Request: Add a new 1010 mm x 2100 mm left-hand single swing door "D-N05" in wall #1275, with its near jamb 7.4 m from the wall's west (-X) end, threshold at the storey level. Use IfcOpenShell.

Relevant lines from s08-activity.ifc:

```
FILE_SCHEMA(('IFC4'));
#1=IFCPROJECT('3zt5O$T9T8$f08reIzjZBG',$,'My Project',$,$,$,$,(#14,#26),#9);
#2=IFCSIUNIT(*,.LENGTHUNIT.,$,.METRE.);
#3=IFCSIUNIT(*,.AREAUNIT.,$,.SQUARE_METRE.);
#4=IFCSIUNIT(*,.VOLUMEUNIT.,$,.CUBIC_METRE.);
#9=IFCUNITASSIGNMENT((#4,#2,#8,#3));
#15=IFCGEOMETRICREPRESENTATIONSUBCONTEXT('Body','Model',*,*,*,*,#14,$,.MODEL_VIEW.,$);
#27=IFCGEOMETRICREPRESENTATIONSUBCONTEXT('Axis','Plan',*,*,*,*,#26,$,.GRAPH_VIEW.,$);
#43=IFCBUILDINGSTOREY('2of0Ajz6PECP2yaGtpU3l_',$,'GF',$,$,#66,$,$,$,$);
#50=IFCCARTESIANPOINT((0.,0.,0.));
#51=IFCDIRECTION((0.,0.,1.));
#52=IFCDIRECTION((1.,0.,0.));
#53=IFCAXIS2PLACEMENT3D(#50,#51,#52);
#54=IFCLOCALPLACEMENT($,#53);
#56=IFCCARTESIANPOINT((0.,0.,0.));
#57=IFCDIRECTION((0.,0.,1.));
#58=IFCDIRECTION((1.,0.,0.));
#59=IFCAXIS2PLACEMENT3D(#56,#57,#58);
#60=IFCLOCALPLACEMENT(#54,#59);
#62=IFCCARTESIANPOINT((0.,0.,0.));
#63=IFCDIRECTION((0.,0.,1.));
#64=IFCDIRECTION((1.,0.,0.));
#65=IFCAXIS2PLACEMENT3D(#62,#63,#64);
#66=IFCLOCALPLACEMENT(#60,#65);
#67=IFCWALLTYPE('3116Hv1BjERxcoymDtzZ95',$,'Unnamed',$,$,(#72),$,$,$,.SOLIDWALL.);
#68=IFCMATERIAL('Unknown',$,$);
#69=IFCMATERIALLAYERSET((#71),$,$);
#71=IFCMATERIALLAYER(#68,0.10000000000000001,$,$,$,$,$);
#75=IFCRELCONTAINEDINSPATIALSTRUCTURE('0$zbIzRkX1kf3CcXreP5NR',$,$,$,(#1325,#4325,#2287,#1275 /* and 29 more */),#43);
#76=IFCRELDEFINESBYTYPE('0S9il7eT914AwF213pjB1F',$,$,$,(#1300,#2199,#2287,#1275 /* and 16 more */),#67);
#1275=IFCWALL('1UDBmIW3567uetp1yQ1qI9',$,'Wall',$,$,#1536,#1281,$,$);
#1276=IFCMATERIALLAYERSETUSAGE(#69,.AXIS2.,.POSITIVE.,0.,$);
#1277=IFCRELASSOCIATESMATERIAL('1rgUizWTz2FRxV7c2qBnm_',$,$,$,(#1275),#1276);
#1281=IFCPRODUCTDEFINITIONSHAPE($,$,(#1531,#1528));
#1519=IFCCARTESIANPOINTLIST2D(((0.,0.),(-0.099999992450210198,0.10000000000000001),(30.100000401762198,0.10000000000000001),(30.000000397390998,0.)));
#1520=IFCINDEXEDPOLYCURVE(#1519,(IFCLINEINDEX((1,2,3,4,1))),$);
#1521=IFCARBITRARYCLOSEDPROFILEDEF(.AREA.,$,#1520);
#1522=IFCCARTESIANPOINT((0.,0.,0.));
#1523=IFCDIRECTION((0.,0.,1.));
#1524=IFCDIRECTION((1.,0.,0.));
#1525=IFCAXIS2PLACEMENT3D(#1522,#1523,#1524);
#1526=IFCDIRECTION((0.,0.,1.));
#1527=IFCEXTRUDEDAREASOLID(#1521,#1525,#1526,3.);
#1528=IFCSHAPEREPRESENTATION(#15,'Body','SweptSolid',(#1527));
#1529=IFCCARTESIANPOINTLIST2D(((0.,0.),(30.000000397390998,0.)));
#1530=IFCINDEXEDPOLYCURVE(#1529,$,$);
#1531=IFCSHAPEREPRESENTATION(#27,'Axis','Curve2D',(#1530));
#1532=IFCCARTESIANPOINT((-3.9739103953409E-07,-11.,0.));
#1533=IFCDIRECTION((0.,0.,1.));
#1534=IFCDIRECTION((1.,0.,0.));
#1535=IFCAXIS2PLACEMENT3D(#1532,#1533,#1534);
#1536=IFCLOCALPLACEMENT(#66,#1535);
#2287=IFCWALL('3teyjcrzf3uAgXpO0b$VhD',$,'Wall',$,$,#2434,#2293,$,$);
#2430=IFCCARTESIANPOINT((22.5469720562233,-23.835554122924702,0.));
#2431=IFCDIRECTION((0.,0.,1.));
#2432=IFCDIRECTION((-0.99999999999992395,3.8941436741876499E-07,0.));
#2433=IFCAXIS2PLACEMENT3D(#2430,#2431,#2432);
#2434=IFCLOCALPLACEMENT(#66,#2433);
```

```python
import numpy as np
import ifcopenshell
import ifcopenshell.api.feature
import ifcopenshell.api.geometry
import ifcopenshell.api.root
import ifcopenshell.api.spatial
import ifcopenshell.geom
import ifcopenshell.util.element
import ifcopenshell.util.placement
import ifcopenshell.util.representation
import ifcopenshell.util.shape
import ifcopenshell.util.unit

model = ifcopenshell.open("s08-activity.ifc")
unit_scale = ifcopenshell.util.unit.calculate_unit_scale(model)
settings = ifcopenshell.geom.settings()


def volume(element):
    """Net volume in cubic metres, openings subtracted."""
    shape = ifcopenshell.geom.create_shape(settings, element)
    return ifcopenshell.util.shape.get_volume(shape.geometry)


wall = model.by_guid("1UDBmIW3567uetp1yQ1qI9")
storey = ifcopenshell.util.element.get_container(wall, ifc_class="IfcBuildingStorey")
context = ifcopenshell.util.representation.get_context(model, "Model", "Body", "MODEL_VIEW")
before = volume(wall)

width, height, from_end, sill = 1.01, 2.1, 7.4, 0.0  # metres

# The wall runs along its own X axis, and the end named is its -X end.
wall_shape = ifcopenshell.geom.create_shape(settings, wall)
x, y, z = ifcopenshell.util.shape.get_vertices(wall_shape.geometry).T
start = x.min() + from_end
face, thickness = float(y.min()), float(y.max() - y.min())
wall_matrix = ifcopenshell.util.placement.get_local_placement(wall.ObjectPlacement)
level = ifcopenshell.util.placement.get_local_placement(storey.ObjectPlacement)[2, 3]


def in_wall(x, y):
    """Placement at x, y metres in the wall's axes, at sill height."""
    matrix = wall_matrix.copy()
    matrix[:, 3] = wall_matrix @ np.array([x / unit_scale, y / unit_scale, 0.0, 1.0])
    matrix[2, 3] = level + sill / unit_scale
    return matrix


# Opening: a box that overshoots both wall faces by 50 mm.
opening = ifcopenshell.api.root.create_entity(model, ifc_class="IfcOpeningElement", predefined_type="OPENING")
box = ifcopenshell.api.geometry.add_wall_representation(
    model, context=context, length=width, height=height, thickness=thickness + 0.1
)
ifcopenshell.api.geometry.assign_representation(model, product=opening, representation=box)
ifcopenshell.api.geometry.edit_object_placement(model, product=opening, matrix=in_wall(start, face - 0.05), is_si=False)
ifcopenshell.api.feature.add_feature(model, feature=opening, element=wall)

door = ifcopenshell.api.root.create_entity(model, ifc_class="IfcDoor", name="D-N05", predefined_type="DOOR")
door.OverallWidth, door.OverallHeight = width / unit_scale, height / unit_scale
door.OperationType = "SINGLE_SWING_LEFT"
body = ifcopenshell.api.geometry.add_door_representation(
    model,
    context=context,
    overall_width=door.OverallWidth,
    overall_height=door.OverallHeight,
    operation_type="SINGLE_SWING_LEFT",
    lining_properties={"LiningDepth": thickness / unit_scale, "ThresholdDepth": thickness / unit_scale},
)
ifcopenshell.api.geometry.assign_representation(model, product=door, representation=body)
ifcopenshell.api.spatial.assign_container(model, products=[door], relating_structure=storey)
ifcopenshell.api.feature.add_filling(model, opening=opening, element=door)

# The lining spans the wall, so the door starts at the wall face.
ifcopenshell.api.geometry.edit_object_placement(model, product=door, matrix=in_wall(start, face), is_si=False)

after = volume(wall)

print(f"wall volume {before:.3f} -> {after:.3f} m3")

model.write("s08-activity_edited.ifc")
```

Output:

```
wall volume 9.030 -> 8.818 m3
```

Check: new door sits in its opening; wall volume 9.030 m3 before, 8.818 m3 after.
